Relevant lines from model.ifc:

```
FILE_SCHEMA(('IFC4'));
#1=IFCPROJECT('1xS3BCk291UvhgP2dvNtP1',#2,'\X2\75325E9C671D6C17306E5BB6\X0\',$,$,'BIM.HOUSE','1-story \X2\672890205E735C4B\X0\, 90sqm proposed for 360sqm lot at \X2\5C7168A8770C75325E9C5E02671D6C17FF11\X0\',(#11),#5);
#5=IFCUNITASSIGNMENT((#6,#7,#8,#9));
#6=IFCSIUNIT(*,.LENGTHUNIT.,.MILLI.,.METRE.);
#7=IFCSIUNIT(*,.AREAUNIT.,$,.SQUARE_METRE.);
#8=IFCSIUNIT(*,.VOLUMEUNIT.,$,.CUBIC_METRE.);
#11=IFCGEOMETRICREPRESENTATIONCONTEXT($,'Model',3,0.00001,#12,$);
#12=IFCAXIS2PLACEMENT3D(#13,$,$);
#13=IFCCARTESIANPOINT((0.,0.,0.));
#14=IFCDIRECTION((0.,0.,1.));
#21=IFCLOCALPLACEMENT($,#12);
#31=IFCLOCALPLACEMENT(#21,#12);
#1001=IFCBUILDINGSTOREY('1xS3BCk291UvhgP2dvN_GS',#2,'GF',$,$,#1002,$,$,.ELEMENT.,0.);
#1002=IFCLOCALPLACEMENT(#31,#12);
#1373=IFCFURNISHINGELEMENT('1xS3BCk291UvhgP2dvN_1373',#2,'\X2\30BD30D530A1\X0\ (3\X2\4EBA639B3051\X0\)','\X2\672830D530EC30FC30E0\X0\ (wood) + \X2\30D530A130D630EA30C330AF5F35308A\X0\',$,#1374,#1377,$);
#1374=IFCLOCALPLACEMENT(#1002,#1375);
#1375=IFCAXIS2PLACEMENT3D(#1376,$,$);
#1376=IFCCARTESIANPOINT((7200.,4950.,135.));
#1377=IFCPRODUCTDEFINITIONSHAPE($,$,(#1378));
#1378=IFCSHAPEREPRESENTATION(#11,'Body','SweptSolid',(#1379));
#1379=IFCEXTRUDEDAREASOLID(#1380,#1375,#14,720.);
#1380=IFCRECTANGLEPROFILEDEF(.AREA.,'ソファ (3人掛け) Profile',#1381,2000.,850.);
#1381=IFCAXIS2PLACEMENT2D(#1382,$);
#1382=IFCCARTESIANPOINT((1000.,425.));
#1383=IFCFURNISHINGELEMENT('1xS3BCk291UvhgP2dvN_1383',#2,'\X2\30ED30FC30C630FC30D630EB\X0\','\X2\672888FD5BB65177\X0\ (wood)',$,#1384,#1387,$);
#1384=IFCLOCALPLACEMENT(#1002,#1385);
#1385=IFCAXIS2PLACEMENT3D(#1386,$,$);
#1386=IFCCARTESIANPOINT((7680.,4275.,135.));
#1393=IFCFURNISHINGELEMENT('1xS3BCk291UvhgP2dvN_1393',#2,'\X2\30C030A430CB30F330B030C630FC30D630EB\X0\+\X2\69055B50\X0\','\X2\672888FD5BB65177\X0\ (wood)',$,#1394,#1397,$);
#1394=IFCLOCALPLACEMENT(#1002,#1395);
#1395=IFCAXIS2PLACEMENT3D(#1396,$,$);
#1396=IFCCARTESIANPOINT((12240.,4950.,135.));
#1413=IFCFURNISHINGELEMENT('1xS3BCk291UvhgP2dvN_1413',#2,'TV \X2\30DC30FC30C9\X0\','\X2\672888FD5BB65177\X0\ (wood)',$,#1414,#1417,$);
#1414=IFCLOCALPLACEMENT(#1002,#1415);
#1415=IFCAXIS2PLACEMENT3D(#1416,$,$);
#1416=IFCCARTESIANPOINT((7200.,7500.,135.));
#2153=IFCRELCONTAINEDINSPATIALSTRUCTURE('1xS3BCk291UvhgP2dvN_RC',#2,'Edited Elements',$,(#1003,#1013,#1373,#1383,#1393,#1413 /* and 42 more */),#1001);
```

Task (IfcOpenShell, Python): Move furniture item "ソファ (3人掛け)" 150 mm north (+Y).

```python
import ifcopenshell
import ifcopenshell.api.geometry
import ifcopenshell.util.placement

model = ifcopenshell.open("model.ifc")

item = model.by_guid("1xS3BCk291UvhgP2dvN_1373")
matrix = ifcopenshell.util.placement.get_local_placement(item.ObjectPlacement)
matrix[1, 3] += 150.0
ifcopenshell.api.geometry.edit_object_placement(model, product=item, matrix=matrix, is_si=False)

print(ifcopenshell.util.placement.get_local_placement(item.ObjectPlacement).round(3) + 0.0)

model.write("model-out.ifc")
```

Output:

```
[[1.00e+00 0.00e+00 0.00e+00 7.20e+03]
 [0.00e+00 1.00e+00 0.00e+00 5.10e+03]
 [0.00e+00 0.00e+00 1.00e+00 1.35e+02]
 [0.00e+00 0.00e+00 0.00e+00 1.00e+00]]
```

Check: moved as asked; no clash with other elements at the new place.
